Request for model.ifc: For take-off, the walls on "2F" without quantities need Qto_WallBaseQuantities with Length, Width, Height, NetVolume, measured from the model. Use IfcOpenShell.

First a look at what the model holds.

```python
import ifcopenshell
import ifcopenshell.util.element
import ifcopenshell.util.unit

model = ifcopenshell.open("model.ifc")
print(model.schema)
for unit_type in ("LENGTHUNIT", "AREAUNIT", "VOLUMEUNIT"):
    print(unit_type, ifcopenshell.util.unit.calculate_unit_scale(model, unit_type))
storey = next(s for s in model.by_type("IfcBuildingStorey") if s.Name == "2F")
walls = [e for e in ifcopenshell.util.element.get_decomposition(storey) if e.is_a("IfcWall")]
for e in sorted(walls, key=lambda e: e.id()):
    print(e.id(), e.is_a(), e.Name, list(ifcopenshell.util.element.get_psets(e, qtos_only=True)), sep=" | ")
```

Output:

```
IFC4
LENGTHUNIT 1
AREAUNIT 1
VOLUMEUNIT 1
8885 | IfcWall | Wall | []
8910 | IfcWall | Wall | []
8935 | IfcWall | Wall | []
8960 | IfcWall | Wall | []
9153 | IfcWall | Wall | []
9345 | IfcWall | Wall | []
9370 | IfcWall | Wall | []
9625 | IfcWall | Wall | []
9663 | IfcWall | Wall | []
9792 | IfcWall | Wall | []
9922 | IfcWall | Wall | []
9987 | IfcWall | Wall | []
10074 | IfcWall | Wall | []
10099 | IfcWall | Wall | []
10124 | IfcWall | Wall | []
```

```python
import ifcopenshell
import ifcopenshell.api.pset
import ifcopenshell.geom
import ifcopenshell.util.element
import ifcopenshell.util.shape
import ifcopenshell.util.unit

model = ifcopenshell.open("model.ifc")
unit_scale = ifcopenshell.util.unit.calculate_unit_scale(model)
volume_scale = ifcopenshell.util.unit.calculate_unit_scale(model, "VOLUMEUNIT")
settings = ifcopenshell.geom.settings()

storey = next(s for s in model.by_type("IfcBuildingStorey") if s.Name == "2F")
walls = [e for e in ifcopenshell.util.element.get_decomposition(storey) if e.is_a("IfcWall")]

for e in sorted(walls, key=lambda e: e.id()):
    if ifcopenshell.util.element.get_psets(e, qtos_only=True, should_inherit=False):
        continue
    # Geometry comes back in metres, in the element's own axes.
    shape = ifcopenshell.geom.create_shape(settings, e)
    values = {
        "Length": ifcopenshell.util.shape.get_x(shape.geometry) / unit_scale,
        "Width": ifcopenshell.util.shape.get_y(shape.geometry) / unit_scale,
        "Height": ifcopenshell.util.shape.get_z(shape.geometry) / unit_scale,
        "NetVolume": ifcopenshell.util.shape.get_volume(shape.geometry) / volume_scale,
    }
    qto = ifcopenshell.api.pset.add_qto(model, product=e, name="Qto_WallBaseQuantities")
    ifcopenshell.api.pset.edit_qto(model, qto=qto, properties=values)
    print(e.id(), {k: round(v, 3) for k, v in values.items()})

model.write("model_rev.ifc")
```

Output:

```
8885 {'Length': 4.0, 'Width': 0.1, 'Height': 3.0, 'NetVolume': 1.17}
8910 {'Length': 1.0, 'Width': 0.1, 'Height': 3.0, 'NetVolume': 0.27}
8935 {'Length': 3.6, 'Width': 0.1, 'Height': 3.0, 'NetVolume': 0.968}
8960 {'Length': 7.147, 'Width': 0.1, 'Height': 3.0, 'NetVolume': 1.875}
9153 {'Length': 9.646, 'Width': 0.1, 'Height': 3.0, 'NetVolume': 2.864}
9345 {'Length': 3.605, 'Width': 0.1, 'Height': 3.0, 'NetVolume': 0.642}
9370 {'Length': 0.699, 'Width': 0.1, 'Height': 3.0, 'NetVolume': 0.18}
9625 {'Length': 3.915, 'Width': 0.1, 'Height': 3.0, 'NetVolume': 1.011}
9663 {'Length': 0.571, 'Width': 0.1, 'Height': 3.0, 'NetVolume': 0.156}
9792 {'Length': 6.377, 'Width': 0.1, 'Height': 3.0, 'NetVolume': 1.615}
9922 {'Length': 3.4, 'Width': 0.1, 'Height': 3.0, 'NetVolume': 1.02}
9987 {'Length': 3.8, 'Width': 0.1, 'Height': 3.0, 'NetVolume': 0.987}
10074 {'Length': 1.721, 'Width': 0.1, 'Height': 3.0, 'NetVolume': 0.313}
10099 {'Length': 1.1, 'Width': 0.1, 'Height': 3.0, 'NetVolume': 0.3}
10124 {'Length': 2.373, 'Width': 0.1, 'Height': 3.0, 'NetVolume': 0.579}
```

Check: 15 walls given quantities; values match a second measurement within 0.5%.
